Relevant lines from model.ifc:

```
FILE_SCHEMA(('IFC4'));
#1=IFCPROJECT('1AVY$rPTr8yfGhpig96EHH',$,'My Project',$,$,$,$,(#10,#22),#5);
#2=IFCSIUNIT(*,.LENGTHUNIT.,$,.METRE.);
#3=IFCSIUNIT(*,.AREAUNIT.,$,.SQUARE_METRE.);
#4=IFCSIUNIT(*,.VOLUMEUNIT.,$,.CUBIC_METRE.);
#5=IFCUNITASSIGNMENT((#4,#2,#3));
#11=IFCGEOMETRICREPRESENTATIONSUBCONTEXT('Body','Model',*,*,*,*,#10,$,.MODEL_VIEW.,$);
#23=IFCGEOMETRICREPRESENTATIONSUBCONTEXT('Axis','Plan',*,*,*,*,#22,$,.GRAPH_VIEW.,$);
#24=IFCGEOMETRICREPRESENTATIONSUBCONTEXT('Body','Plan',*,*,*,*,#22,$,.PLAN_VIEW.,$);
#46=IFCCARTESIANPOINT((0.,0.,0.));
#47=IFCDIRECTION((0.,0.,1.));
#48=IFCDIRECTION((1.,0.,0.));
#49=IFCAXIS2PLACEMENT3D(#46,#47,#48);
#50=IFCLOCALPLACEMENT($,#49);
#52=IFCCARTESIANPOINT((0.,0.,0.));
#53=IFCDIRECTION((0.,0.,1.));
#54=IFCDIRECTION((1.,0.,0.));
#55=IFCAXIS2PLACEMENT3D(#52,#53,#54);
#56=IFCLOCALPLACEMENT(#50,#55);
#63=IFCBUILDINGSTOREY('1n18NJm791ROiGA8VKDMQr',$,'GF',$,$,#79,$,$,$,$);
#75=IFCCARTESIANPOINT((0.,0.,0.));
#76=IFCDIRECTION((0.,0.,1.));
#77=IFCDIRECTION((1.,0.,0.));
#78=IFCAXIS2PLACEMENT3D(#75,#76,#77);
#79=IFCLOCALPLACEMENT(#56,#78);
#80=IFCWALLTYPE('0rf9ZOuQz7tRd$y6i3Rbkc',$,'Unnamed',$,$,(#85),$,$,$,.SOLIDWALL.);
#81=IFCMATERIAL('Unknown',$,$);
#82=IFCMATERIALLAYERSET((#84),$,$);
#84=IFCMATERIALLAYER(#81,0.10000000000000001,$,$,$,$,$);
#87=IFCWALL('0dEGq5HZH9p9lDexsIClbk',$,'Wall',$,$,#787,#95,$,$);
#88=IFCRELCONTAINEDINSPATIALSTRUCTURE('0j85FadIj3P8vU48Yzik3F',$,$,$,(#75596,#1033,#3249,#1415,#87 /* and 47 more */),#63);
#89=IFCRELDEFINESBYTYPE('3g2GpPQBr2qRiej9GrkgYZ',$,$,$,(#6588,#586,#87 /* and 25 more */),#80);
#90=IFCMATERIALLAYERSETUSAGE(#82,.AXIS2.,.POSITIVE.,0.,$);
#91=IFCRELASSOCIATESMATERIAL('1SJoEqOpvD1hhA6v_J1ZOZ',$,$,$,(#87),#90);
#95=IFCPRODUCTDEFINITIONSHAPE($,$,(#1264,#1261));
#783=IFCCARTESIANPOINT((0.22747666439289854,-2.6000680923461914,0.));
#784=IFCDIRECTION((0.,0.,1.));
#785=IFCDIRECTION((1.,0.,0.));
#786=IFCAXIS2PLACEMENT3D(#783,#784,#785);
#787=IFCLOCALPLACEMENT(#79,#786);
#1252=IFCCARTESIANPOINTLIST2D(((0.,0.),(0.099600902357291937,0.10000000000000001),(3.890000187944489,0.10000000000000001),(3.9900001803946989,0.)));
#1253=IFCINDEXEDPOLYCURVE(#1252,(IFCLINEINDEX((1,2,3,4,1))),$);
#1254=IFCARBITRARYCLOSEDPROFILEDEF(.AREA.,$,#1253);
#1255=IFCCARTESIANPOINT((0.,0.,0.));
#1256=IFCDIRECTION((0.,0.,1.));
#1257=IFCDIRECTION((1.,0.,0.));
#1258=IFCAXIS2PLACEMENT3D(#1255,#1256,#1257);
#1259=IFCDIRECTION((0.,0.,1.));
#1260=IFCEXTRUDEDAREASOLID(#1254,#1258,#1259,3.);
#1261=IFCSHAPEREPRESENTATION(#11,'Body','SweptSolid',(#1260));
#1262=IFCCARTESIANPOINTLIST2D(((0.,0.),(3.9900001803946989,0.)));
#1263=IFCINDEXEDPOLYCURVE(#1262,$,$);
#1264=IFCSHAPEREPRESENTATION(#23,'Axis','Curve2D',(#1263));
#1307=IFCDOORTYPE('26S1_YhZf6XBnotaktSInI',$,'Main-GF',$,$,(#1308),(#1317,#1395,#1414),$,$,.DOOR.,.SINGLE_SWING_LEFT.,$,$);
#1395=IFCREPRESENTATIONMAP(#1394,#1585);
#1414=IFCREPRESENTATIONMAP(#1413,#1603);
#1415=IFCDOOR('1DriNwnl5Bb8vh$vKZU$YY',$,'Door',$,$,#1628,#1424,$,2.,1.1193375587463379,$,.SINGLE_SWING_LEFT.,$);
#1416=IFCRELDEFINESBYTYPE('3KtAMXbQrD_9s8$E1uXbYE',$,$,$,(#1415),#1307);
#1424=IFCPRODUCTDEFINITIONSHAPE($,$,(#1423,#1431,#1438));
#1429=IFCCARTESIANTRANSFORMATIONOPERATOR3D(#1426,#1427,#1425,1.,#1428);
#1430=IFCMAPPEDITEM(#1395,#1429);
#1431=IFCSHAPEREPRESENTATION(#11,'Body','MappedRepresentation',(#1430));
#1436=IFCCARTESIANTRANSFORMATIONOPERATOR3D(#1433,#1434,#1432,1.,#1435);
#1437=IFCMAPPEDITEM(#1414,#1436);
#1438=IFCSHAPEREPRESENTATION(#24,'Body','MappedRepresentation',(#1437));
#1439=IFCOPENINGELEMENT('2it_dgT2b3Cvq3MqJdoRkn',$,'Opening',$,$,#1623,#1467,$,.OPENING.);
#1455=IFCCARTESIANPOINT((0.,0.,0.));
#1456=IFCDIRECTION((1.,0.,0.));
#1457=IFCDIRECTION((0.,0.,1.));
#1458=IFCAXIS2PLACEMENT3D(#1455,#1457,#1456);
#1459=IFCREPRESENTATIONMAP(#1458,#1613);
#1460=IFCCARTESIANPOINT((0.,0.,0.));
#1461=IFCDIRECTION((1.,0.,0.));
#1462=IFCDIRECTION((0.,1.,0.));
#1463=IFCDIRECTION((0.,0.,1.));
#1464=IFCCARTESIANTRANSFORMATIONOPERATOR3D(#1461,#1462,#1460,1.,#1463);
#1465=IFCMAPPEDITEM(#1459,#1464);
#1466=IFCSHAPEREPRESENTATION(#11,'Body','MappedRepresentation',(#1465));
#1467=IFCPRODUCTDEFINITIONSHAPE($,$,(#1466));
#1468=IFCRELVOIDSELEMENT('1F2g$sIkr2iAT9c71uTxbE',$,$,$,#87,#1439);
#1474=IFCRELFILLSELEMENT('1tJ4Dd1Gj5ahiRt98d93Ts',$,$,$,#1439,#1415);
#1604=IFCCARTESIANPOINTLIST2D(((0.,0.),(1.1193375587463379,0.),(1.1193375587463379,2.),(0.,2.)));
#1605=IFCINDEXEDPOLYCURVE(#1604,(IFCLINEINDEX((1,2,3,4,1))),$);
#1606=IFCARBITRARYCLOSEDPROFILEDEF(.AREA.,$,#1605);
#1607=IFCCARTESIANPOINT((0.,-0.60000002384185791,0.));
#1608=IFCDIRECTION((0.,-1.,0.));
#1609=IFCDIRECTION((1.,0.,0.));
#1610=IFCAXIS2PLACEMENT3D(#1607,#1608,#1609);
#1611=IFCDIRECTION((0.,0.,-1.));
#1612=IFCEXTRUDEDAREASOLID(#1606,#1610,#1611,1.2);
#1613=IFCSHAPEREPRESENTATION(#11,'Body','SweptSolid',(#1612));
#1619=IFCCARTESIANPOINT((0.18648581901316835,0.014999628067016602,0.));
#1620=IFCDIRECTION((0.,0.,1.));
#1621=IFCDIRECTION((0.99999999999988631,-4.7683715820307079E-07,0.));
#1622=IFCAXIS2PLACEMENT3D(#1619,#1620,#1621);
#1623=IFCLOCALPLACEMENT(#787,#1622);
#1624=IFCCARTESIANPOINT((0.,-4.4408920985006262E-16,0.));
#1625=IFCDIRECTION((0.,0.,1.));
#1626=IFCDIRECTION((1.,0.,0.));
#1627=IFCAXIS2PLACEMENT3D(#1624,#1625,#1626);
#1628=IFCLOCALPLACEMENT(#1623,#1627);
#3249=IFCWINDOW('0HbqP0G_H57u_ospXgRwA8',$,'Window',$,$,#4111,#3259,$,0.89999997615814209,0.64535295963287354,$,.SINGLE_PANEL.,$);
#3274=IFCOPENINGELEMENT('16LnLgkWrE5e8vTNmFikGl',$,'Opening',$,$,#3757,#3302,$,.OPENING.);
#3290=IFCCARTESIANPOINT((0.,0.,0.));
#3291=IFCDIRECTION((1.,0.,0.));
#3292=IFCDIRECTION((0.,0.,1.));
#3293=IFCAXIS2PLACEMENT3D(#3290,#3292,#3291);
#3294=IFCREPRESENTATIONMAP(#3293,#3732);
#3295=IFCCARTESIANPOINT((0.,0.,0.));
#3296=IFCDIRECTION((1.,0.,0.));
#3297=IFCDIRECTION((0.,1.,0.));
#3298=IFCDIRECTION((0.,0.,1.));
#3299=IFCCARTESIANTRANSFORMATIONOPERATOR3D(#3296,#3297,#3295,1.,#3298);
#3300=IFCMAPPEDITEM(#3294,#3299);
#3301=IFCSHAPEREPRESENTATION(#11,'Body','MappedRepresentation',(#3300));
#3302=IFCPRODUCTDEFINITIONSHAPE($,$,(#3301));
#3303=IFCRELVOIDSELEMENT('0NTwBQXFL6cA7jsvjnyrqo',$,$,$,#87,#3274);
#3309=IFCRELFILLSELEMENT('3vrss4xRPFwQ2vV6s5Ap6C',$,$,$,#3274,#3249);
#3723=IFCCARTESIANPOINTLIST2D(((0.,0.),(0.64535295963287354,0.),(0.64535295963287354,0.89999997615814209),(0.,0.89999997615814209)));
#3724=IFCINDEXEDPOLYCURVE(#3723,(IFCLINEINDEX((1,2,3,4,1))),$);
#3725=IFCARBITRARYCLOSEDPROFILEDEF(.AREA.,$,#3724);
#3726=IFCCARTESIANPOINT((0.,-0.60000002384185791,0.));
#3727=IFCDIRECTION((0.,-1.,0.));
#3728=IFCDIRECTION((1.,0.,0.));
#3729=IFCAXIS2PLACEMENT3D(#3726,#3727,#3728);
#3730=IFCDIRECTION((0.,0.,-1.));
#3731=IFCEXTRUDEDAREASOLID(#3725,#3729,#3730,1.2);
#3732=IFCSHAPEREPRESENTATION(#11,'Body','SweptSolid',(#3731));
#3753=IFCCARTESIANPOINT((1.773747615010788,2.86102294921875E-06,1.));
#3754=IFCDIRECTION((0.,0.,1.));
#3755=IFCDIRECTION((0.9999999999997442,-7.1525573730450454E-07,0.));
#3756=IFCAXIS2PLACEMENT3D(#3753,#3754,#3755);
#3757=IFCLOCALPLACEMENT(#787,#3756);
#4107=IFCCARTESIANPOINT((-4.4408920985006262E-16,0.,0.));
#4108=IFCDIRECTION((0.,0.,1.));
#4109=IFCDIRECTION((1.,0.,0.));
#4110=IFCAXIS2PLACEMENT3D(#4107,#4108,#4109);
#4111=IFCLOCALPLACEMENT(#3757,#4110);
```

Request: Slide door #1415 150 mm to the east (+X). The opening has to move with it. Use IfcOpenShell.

```python
import ifcopenshell
import ifcopenshell.api.geometry
import ifcopenshell.util.placement

model = ifcopenshell.open("model.ifc")

door = model.by_guid("1DriNwnl5Bb8vh$vKZU$YY")
opening = door.FillsVoids[0].RelatingOpeningElement
wall = opening.VoidsElements[0].RelatingBuildingElement

wall_matrix = ifcopenshell.util.placement.get_local_placement(wall.ObjectPlacement)
shift = wall_matrix[:3, 0] * 0.15
before = ifcopenshell.util.placement.get_local_placement(door.ObjectPlacement)[:3, 3].copy()

# The door is placed relative to its opening, so it follows when the opening moves.
matrix = ifcopenshell.util.placement.get_local_placement(opening.ObjectPlacement)
matrix[:3, 3] += shift
ifcopenshell.api.geometry.edit_object_placement(
    model, product=opening, matrix=matrix, is_si=False, should_transform_children=True
)

after = ifcopenshell.util.placement.get_local_placement(door.ObjectPlacement)[:3, 3]
print("door moved by", (after - before).round(3) + 0.0)

model.write("model-out.ifc")
```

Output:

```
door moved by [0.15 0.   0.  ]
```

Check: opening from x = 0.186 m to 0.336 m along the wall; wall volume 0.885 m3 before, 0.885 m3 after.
